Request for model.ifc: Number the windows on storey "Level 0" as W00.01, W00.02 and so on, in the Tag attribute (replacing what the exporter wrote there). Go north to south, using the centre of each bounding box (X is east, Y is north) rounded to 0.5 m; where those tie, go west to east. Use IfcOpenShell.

First a look at what the model holds.

```python
import ifcopenshell
import ifcopenshell.util.element
import ifcopenshell.util.placement

model = ifcopenshell.open("model.ifc")
print(model.schema)
storey = next(s for s in model.by_type("IfcBuildingStorey") if s.Name == "Level 0")
windows = [e for e in ifcopenshell.util.element.get_decomposition(storey) if e.is_a("IfcWindow")]
for e in sorted(windows, key=lambda e: e.id()):
    origin = ifcopenshell.util.placement.get_local_placement(e.ObjectPlacement)[:3, 3]
    print(e.id(), e.Tag, e.Name, origin.round(2) + 0.0, sep=" | ")
```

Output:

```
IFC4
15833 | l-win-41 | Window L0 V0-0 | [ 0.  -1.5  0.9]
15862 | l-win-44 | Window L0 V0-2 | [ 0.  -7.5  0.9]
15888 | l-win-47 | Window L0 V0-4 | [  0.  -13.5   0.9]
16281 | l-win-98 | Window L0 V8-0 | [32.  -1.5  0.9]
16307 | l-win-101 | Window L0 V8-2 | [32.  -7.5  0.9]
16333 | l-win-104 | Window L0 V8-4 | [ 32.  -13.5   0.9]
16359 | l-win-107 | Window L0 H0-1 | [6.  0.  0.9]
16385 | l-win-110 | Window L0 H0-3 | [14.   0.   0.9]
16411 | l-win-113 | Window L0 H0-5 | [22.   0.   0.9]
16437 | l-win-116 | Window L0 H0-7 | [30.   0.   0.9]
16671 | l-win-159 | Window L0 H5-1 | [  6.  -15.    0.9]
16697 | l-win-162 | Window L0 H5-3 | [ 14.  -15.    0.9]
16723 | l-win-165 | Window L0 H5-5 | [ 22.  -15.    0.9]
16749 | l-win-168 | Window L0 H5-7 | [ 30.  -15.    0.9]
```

```python
import ifcopenshell
import ifcopenshell.geom
import ifcopenshell.util.element
import ifcopenshell.util.shape

model = ifcopenshell.open("model.ifc")
settings = ifcopenshell.geom.settings()
settings.set("use-world-coords", True)


def centre(element):
    shape = ifcopenshell.geom.create_shape(settings, element)
    return ifcopenshell.util.shape.get_bbox_centroid(shape.geometry)


storey = next(s for s in model.by_type("IfcBuildingStorey") if s.Name == "Level 0")
windows = [e for e in ifcopenshell.util.element.get_decomposition(storey) if e.is_a("IfcWindow")]

# Insertion points can sit at a corner or the storey origin, so sort by the geometry (in metres).
centres = {e: centre(e) for e in windows}
windows.sort(key=lambda e: (-round(centres[e][1] / 0.5), centres[e][0]))

for i, e in enumerate(windows, start=1):
    number = f"W00.{i:02d}"
    e.Tag = number
    print(e.id(), number)

model.write("model_updated.ifc")
```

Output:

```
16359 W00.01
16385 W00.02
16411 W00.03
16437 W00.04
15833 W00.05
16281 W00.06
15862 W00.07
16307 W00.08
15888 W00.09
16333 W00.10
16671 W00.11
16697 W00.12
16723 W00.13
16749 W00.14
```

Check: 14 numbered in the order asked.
